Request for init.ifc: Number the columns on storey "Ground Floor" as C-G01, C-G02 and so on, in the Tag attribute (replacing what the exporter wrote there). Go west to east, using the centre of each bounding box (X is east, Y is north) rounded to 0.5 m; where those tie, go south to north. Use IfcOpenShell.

First a look at what the model holds.

```python
import ifcopenshell
import ifcopenshell.util.element
import ifcopenshell.util.placement

model = ifcopenshell.open("init.ifc")
print(model.schema)
storey = next(s for s in model.by_type("IfcBuildingStorey") if s.Name == "Ground Floor")
columns = [e for e in ifcopenshell.util.element.get_decomposition(storey) if e.is_a("IfcColumn")]
for e in sorted(columns, key=lambda e: e.id()):
    origin = ifcopenshell.util.placement.get_local_placement(e.ObjectPlacement)[:3, 3]
    print(e.id(), e.Tag, e.Name, origin.round(2) + 0.0, sep=" | ")
```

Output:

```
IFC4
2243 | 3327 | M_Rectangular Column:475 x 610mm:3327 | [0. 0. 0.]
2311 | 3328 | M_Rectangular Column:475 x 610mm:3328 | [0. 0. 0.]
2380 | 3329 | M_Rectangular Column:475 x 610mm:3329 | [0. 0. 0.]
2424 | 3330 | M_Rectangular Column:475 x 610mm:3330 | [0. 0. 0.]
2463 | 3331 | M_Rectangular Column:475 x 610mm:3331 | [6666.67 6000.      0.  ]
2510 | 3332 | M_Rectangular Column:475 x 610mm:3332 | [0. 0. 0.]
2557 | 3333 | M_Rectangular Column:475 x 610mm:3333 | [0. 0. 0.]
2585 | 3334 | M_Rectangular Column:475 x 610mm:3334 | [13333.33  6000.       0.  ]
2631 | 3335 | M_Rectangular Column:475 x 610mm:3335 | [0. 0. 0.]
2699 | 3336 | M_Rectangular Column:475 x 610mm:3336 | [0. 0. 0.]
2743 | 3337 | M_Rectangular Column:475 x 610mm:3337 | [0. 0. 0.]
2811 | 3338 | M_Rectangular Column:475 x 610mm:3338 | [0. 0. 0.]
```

```python
import ifcopenshell
import ifcopenshell.geom
import ifcopenshell.util.element
import ifcopenshell.util.shape

model = ifcopenshell.open("init.ifc")
settings = ifcopenshell.geom.settings()
settings.set("use-world-coords", True)


def centre(element):
    shape = ifcopenshell.geom.create_shape(settings, element)
    return ifcopenshell.util.shape.get_bbox_centroid(shape.geometry)


storey = next(s for s in model.by_type("IfcBuildingStorey") if s.Name == "Ground Floor")
columns = [e for e in ifcopenshell.util.element.get_decomposition(storey) if e.is_a("IfcColumn")]

# Insertion points can sit at a corner or the storey origin, so sort by the geometry (in metres).
centres = {e: centre(e) for e in columns}
columns.sort(key=lambda e: (round(centres[e][0] / 0.5), centres[e][1]))

for i, e in enumerate(columns, start=1):
    number = f"C-G{i:02d}"
    e.Tag = number
    print(e.id(), number)

model.write("init_rev.ifc")
```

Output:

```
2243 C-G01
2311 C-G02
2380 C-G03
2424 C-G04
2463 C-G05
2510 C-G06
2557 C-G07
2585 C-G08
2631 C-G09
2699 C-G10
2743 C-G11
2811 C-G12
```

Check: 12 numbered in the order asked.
